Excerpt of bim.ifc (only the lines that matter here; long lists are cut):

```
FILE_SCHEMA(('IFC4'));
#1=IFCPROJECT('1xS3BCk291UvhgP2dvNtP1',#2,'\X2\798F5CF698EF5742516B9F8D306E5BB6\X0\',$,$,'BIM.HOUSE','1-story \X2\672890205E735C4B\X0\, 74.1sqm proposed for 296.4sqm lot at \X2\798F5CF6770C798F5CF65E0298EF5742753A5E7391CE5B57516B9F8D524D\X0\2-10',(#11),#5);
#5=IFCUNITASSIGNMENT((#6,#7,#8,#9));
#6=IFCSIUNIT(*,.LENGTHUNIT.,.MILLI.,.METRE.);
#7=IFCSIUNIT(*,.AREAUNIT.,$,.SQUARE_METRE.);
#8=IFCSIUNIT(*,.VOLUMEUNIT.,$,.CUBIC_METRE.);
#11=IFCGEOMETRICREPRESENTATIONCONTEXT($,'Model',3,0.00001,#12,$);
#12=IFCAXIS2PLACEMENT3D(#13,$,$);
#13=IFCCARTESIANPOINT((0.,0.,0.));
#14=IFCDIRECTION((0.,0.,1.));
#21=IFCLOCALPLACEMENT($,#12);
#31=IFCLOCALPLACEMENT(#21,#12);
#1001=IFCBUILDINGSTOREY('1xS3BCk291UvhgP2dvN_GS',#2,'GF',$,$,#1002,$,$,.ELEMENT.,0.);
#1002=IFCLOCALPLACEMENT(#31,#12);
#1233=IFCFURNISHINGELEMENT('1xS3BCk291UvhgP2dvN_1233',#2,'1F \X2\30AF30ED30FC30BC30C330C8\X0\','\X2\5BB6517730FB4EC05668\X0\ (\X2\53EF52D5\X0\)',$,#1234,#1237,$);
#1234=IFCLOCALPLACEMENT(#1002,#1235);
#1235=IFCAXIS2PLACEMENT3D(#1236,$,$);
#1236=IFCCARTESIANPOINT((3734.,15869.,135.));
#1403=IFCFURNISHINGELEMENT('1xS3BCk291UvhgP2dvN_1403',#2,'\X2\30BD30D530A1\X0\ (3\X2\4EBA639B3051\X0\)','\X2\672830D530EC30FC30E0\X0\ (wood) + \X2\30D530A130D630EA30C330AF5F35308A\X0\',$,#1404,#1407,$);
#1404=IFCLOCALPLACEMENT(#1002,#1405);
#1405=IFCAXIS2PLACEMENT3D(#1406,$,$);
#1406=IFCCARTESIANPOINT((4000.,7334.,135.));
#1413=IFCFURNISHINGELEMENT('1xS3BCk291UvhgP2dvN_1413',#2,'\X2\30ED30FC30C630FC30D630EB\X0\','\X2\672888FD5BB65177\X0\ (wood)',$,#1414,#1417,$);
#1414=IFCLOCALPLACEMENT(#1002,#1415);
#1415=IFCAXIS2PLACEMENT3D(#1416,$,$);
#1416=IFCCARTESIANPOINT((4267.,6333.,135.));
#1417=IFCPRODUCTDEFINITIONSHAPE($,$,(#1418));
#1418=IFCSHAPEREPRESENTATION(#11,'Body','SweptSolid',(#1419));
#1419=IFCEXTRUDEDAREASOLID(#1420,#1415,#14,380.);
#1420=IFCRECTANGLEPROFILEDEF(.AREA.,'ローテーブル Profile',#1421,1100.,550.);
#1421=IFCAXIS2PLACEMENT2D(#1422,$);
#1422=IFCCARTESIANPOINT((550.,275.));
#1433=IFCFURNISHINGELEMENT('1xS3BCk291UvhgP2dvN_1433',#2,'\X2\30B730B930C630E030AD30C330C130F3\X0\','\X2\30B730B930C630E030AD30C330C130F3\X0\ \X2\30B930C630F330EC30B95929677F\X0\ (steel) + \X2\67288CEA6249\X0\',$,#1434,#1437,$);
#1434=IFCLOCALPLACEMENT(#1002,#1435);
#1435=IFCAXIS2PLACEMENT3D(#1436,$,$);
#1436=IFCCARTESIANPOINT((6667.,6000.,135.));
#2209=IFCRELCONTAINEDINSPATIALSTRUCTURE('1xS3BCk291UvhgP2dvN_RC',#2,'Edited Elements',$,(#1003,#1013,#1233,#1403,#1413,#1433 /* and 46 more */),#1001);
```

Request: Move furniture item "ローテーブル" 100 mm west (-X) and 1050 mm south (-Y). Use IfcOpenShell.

```python
import ifcopenshell
import ifcopenshell.api.geometry
import ifcopenshell.util.placement

model = ifcopenshell.open("bim.ifc")

item = model.by_guid("1xS3BCk291UvhgP2dvN_1413")
matrix = ifcopenshell.util.placement.get_local_placement(item.ObjectPlacement)
matrix[0, 3] -= 100.0
matrix[1, 3] -= 1050.0
ifcopenshell.api.geometry.edit_object_placement(model, product=item, matrix=matrix, is_si=False)

print(ifcopenshell.util.placement.get_local_placement(item.ObjectPlacement).round(3) + 0.0)

model.write("bim_v2.ifc")
```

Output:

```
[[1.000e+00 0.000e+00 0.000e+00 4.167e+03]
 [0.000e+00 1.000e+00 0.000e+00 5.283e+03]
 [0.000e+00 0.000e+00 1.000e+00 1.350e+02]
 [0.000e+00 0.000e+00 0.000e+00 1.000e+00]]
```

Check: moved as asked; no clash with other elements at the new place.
